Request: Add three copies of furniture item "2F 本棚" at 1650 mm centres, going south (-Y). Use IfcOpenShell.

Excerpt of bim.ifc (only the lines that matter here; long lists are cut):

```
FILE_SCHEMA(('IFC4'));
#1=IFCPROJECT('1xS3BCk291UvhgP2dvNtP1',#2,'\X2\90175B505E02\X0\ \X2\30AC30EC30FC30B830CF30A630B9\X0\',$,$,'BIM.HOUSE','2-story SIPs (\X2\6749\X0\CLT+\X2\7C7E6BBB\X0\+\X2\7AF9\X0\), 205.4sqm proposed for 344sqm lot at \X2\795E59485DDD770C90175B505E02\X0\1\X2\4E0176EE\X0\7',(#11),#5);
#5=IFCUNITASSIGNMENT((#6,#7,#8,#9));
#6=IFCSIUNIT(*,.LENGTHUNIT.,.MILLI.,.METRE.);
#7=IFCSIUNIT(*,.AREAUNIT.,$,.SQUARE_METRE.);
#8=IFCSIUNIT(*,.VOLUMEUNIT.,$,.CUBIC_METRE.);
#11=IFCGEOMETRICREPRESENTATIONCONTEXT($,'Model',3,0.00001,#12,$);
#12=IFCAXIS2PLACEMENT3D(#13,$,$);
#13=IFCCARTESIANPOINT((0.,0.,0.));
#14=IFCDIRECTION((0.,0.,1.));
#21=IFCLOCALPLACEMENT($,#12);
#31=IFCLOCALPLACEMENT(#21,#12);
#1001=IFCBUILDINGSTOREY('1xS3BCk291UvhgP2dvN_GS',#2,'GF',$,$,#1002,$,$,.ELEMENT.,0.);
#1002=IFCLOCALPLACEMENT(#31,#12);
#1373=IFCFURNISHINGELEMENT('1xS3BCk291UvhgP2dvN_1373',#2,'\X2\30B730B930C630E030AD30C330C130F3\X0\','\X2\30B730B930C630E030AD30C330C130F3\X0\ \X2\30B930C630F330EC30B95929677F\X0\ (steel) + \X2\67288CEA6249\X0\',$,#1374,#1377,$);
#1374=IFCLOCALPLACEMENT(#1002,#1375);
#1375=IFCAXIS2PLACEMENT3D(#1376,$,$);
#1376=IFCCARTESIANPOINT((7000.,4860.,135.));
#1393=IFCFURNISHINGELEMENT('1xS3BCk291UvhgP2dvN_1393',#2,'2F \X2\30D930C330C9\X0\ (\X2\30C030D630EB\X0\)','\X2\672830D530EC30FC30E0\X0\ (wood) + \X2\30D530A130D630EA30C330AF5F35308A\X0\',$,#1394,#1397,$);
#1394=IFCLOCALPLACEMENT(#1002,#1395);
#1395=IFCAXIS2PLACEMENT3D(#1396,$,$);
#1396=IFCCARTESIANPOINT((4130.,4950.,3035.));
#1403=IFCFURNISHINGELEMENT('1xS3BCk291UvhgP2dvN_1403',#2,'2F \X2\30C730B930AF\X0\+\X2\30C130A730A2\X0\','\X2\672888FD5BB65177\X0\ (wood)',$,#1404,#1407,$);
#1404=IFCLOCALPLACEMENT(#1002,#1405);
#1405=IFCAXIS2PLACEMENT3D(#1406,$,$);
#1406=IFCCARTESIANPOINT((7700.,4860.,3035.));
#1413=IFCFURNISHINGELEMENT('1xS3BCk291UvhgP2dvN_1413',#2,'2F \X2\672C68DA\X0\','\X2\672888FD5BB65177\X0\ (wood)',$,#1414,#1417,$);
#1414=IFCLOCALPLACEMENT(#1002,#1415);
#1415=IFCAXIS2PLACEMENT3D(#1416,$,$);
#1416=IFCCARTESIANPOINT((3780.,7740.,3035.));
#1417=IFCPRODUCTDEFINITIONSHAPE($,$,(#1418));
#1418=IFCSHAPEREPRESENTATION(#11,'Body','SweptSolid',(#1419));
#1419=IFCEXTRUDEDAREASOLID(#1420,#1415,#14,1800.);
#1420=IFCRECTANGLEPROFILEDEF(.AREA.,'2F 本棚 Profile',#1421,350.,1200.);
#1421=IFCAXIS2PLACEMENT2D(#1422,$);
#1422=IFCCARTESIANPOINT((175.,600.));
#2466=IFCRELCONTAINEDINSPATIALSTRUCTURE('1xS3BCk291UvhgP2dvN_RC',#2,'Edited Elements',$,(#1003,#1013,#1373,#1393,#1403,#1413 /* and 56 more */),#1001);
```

```python
import numpy as np
import ifcopenshell
import ifcopenshell.api.geometry
import ifcopenshell.api.root
import ifcopenshell.util.element
import ifcopenshell.util.placement
import ifcopenshell.util.unit

model = ifcopenshell.open("bim.ifc")
unit_scale = ifcopenshell.util.unit.calculate_unit_scale(model)


def reuse_history(source, copy):
    """copy_class also copies each property set's owner history, people and application; keep the originals."""
    for rel in copy.IsDefinedBy:
        if rel.is_a("IfcRelDefinesByProperties") and (history := rel.RelatingPropertyDefinition.OwnerHistory):
            rel.RelatingPropertyDefinition.OwnerHistory = source.OwnerHistory
            ifcopenshell.util.element.remove_deep2(model, history)


source = model.by_id(1413)
base = ifcopenshell.util.placement.get_local_placement(source.ObjectPlacement)
step = np.array([0.0, -1.0, 0.0]) * 1.65 / unit_scale

for i in range(1, 4):
    copy = ifcopenshell.api.root.copy_class(model, product=source)
    copy.Representation = ifcopenshell.util.element.copy_deep(
        model, source.Representation, exclude=["IfcGeometricRepresentationContext", "IfcRepresentationMap"]
    )
    reuse_history(source, copy)
    matrix = base.copy()
    matrix[:3, 3] += i * step
    print("added at", matrix[:3, 3].round(3) + 0.0)
    ifcopenshell.api.geometry.edit_object_placement(model, product=copy, matrix=matrix, is_si=False)

model.write("bim_updated.ifc")
```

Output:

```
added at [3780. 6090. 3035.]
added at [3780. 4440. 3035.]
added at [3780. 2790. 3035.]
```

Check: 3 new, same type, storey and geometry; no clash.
